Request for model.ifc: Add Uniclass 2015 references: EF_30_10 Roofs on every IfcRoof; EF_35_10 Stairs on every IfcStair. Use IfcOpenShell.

First a look at what the model holds.

```python
import ifcopenshell

model = ifcopenshell.open("model.ifc")
print(model.schema)
print("classifications:", [c.Name for c in model.by_type("IfcClassification")])
for ifc_class in ("IfcDoor", "IfcRoof", "IfcStair", "IfcWall", "IfcWindow"):
    print(ifc_class, len(model.by_type(ifc_class)))
```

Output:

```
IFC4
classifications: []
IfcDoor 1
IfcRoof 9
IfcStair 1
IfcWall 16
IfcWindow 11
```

```python
import ifcopenshell
import ifcopenshell.api.classification

model = ifcopenshell.open("model.ifc")

system = ifcopenshell.api.classification.add_classification(model, classification="Uniclass 2015")

codes = {
    "IfcRoof": ("EF_30_10", "Roofs"),
    "IfcStair": ("EF_35_10", "Stairs"),
}
for ifc_class, (code, name) in codes.items():
    products = model.by_type(ifc_class)
    ifcopenshell.api.classification.add_reference(
        model, products=products, classification=system, identification=code, name=name
    )
    print(code, len(products))

model.write("model-out.ifc")
```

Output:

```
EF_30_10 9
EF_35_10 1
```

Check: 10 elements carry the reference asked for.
